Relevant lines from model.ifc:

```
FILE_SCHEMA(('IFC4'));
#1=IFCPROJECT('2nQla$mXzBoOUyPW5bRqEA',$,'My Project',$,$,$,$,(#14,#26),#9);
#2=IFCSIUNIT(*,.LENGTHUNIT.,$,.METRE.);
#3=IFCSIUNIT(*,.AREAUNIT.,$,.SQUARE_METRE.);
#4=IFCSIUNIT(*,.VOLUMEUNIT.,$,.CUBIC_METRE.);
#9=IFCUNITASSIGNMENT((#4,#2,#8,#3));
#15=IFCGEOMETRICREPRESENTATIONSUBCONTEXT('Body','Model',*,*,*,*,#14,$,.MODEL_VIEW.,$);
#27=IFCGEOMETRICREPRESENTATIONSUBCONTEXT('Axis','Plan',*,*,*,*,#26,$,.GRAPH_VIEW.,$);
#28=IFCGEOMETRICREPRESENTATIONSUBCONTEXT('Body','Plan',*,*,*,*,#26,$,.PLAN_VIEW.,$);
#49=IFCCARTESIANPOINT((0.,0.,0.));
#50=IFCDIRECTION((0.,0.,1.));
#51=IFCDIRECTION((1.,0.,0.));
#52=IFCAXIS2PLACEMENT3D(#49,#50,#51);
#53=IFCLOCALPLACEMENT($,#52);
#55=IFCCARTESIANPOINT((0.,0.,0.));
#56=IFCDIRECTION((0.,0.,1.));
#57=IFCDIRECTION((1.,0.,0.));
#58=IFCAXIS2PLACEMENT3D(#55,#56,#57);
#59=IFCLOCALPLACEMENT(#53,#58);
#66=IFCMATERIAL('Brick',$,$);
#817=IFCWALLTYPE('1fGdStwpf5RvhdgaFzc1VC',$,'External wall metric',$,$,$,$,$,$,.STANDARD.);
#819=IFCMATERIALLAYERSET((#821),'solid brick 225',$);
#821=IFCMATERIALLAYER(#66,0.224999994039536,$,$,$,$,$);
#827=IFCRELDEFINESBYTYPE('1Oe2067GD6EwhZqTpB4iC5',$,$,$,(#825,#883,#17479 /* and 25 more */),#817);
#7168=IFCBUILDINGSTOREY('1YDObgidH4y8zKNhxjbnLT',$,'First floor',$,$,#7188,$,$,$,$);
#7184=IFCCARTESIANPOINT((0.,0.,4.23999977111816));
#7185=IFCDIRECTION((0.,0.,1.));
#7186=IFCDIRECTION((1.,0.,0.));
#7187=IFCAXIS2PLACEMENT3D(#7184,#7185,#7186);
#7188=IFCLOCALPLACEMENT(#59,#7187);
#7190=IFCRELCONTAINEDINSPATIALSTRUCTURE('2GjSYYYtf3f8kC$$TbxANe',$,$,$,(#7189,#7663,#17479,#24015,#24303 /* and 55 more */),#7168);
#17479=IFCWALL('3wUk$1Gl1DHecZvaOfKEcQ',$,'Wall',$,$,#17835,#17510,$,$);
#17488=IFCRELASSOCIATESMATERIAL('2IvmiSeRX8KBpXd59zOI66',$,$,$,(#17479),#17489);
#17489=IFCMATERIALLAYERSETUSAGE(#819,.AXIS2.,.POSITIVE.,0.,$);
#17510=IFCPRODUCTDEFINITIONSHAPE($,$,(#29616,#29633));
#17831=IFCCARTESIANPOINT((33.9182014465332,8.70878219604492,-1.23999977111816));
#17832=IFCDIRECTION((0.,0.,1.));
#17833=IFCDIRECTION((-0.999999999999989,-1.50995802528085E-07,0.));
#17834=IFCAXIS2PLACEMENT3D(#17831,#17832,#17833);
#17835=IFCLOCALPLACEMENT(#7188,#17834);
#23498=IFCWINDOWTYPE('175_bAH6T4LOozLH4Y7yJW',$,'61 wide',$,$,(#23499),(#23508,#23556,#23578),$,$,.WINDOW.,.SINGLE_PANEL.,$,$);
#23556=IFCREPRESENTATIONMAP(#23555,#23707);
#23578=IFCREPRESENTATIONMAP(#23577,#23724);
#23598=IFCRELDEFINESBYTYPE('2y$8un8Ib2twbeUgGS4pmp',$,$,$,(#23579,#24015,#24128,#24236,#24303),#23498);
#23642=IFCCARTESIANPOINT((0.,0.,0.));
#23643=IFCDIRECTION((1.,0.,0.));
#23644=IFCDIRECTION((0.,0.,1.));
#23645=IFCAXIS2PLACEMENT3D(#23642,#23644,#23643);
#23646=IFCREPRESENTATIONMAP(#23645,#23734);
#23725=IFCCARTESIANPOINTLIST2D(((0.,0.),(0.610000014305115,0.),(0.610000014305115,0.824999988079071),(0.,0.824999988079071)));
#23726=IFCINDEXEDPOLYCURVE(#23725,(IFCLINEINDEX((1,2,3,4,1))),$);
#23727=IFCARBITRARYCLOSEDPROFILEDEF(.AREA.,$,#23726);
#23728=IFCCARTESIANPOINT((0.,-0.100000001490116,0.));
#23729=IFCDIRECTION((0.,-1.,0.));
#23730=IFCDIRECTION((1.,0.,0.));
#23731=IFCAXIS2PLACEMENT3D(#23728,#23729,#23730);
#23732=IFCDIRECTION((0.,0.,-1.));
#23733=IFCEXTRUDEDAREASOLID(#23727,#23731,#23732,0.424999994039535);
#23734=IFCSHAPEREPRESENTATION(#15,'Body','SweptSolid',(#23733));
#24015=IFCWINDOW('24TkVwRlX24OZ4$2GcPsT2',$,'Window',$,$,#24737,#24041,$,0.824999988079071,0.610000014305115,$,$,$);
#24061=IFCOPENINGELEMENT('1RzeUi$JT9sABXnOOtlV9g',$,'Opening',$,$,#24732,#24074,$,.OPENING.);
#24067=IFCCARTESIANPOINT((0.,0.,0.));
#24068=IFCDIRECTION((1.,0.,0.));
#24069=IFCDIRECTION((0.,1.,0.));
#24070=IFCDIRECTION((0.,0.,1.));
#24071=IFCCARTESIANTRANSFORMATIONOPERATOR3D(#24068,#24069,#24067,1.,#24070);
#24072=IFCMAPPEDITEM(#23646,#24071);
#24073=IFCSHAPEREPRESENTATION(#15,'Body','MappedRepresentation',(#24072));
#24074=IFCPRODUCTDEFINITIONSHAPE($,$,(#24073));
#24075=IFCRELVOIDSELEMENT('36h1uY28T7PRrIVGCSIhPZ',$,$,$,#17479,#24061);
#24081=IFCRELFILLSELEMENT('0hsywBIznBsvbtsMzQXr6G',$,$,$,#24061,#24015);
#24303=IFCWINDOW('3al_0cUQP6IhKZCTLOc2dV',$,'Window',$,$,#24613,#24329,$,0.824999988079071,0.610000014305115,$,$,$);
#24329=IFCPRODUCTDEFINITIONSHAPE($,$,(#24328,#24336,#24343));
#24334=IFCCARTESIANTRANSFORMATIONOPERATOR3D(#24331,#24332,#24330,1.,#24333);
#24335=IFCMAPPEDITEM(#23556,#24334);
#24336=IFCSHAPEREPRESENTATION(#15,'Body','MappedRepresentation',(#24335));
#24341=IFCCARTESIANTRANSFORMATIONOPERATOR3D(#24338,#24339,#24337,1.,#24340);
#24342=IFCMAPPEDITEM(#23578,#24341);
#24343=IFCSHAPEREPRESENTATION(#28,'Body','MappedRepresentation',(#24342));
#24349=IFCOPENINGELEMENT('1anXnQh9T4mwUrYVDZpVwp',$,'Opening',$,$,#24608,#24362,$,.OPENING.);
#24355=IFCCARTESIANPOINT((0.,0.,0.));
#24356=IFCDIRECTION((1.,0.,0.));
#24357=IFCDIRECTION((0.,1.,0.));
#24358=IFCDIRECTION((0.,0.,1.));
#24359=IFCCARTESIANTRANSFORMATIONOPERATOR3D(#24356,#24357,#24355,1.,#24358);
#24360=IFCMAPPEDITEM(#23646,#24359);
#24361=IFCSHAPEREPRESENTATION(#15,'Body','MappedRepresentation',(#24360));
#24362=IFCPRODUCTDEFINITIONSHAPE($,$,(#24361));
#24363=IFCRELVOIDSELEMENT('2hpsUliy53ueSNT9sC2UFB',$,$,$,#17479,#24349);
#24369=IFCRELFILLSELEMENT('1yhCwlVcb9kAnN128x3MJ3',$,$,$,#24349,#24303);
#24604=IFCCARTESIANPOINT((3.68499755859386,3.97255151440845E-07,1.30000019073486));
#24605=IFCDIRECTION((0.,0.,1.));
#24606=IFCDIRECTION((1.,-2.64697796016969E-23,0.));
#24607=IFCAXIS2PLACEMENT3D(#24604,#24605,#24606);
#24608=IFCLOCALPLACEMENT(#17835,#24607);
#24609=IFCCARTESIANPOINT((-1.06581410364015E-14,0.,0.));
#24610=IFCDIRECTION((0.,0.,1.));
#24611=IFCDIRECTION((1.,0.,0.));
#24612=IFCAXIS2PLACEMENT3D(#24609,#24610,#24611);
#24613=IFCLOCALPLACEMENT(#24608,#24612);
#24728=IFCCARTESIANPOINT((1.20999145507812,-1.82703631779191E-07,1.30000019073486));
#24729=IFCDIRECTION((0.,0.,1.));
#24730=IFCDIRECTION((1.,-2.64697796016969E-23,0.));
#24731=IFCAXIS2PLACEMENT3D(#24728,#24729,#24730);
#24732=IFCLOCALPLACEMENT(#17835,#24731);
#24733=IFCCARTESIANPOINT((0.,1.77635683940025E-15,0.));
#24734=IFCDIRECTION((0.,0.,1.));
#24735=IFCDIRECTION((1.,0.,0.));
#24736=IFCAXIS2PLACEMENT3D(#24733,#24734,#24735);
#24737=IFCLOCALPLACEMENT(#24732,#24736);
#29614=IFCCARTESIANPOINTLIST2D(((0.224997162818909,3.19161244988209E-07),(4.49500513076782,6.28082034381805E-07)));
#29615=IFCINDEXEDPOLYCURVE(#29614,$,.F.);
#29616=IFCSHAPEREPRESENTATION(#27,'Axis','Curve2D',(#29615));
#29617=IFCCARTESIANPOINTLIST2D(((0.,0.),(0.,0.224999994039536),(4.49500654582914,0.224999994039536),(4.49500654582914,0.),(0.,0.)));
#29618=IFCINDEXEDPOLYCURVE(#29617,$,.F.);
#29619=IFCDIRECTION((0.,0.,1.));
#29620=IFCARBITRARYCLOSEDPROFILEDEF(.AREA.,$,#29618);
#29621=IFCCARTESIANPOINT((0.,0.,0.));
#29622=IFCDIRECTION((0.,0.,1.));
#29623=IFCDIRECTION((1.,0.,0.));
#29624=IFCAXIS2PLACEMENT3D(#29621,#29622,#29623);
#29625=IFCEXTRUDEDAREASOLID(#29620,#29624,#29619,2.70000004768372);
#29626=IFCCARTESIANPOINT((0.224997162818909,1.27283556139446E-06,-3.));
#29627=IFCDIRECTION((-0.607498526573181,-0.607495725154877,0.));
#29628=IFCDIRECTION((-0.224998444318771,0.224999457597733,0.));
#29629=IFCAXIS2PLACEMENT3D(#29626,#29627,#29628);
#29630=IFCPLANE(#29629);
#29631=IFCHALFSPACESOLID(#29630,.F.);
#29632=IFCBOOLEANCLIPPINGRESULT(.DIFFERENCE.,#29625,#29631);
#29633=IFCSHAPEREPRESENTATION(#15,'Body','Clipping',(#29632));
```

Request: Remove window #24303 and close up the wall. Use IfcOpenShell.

```python
import ifcopenshell
import ifcopenshell.api.feature
import ifcopenshell.api.root
import ifcopenshell.geom
import ifcopenshell.util.shape

model = ifcopenshell.open("model.ifc")
settings = ifcopenshell.geom.settings()


def volume(element):
    """Net volume in cubic metres, openings subtracted."""
    shape = ifcopenshell.geom.create_shape(settings, element)
    return ifcopenshell.util.shape.get_volume(shape.geometry)


window = model.by_guid("3al_0cUQP6IhKZCTLOc2dV")
opening = window.FillsVoids[0].RelatingOpeningElement
wall = opening.VoidsElements[0].RelatingBuildingElement
before = volume(wall)

ifcopenshell.api.root.remove_product(model, product=window)
ifcopenshell.api.feature.remove_feature(model, feature=opening)

after = volume(wall)

print(f"wall volume {before:.3f} -> {after:.3f} m3")

model.write("model_rev.ifc")
```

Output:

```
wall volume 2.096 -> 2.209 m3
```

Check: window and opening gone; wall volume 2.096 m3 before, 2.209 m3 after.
